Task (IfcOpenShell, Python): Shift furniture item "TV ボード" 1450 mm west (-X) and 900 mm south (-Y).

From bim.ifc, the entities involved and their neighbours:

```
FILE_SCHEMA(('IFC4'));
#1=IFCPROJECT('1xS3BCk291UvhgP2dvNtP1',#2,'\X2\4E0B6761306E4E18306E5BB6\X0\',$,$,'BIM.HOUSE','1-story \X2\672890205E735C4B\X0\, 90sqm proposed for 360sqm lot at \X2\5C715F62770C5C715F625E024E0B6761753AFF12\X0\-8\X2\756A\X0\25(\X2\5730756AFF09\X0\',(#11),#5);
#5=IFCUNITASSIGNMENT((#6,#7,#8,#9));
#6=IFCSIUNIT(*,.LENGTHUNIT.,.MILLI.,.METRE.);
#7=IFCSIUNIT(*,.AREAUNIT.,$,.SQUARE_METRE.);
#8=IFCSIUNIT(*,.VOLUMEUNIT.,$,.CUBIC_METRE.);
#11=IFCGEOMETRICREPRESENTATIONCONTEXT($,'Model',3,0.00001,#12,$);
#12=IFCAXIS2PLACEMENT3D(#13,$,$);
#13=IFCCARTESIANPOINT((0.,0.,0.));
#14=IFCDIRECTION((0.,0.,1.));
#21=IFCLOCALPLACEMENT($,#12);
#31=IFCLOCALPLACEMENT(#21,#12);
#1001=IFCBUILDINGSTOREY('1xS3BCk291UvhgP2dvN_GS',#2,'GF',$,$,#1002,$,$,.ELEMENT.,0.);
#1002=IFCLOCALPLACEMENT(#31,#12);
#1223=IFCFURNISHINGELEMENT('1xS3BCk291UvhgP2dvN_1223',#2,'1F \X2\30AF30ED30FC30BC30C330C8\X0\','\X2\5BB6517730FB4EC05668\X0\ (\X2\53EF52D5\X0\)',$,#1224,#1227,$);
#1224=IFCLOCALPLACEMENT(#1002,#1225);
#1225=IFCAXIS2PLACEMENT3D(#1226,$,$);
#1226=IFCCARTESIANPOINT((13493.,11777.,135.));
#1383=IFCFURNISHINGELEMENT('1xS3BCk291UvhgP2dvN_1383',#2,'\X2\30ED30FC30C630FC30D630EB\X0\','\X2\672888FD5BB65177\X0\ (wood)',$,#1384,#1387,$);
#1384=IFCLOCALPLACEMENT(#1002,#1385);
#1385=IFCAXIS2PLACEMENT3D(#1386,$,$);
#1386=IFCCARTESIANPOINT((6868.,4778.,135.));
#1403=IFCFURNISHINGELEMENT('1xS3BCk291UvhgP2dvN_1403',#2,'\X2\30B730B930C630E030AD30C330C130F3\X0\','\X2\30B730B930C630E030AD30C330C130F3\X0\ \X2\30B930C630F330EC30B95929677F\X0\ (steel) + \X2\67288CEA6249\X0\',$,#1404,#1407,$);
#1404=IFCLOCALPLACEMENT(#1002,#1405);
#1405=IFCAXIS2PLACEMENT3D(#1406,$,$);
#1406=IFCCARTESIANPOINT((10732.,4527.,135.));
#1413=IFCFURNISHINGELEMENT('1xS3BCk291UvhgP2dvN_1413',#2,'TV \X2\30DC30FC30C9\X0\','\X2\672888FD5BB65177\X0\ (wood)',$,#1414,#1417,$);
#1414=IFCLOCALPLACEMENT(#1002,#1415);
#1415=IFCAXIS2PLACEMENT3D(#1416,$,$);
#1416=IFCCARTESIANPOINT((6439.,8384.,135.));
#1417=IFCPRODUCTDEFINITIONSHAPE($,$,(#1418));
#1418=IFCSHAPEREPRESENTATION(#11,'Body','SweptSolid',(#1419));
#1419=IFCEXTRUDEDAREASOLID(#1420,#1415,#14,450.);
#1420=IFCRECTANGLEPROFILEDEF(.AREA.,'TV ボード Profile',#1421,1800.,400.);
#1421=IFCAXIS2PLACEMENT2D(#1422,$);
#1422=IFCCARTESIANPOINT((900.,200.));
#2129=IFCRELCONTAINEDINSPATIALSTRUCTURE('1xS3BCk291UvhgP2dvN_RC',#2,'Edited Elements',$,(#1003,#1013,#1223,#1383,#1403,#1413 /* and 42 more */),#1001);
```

```python
import ifcopenshell
import ifcopenshell.api.geometry
import ifcopenshell.util.placement
import ifcopenshell.util.unit

model = ifcopenshell.open("bim.ifc")
unit_scale = ifcopenshell.util.unit.calculate_unit_scale(model)

item = model.by_guid("1xS3BCk291UvhgP2dvN_1413")
matrix = ifcopenshell.util.placement.get_local_placement(item.ObjectPlacement)
matrix[0, 3] -= 1.45 / unit_scale
matrix[1, 3] -= 0.9 / unit_scale
ifcopenshell.api.geometry.edit_object_placement(model, product=item, matrix=matrix, is_si=False)

print(ifcopenshell.util.placement.get_local_placement(item.ObjectPlacement).round(3) + 0.0)

model.write("bim_rev.ifc")
```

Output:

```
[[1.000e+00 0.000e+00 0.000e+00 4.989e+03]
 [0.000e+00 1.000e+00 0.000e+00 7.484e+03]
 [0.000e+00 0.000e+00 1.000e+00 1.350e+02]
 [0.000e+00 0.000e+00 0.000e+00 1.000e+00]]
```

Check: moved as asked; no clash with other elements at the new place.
